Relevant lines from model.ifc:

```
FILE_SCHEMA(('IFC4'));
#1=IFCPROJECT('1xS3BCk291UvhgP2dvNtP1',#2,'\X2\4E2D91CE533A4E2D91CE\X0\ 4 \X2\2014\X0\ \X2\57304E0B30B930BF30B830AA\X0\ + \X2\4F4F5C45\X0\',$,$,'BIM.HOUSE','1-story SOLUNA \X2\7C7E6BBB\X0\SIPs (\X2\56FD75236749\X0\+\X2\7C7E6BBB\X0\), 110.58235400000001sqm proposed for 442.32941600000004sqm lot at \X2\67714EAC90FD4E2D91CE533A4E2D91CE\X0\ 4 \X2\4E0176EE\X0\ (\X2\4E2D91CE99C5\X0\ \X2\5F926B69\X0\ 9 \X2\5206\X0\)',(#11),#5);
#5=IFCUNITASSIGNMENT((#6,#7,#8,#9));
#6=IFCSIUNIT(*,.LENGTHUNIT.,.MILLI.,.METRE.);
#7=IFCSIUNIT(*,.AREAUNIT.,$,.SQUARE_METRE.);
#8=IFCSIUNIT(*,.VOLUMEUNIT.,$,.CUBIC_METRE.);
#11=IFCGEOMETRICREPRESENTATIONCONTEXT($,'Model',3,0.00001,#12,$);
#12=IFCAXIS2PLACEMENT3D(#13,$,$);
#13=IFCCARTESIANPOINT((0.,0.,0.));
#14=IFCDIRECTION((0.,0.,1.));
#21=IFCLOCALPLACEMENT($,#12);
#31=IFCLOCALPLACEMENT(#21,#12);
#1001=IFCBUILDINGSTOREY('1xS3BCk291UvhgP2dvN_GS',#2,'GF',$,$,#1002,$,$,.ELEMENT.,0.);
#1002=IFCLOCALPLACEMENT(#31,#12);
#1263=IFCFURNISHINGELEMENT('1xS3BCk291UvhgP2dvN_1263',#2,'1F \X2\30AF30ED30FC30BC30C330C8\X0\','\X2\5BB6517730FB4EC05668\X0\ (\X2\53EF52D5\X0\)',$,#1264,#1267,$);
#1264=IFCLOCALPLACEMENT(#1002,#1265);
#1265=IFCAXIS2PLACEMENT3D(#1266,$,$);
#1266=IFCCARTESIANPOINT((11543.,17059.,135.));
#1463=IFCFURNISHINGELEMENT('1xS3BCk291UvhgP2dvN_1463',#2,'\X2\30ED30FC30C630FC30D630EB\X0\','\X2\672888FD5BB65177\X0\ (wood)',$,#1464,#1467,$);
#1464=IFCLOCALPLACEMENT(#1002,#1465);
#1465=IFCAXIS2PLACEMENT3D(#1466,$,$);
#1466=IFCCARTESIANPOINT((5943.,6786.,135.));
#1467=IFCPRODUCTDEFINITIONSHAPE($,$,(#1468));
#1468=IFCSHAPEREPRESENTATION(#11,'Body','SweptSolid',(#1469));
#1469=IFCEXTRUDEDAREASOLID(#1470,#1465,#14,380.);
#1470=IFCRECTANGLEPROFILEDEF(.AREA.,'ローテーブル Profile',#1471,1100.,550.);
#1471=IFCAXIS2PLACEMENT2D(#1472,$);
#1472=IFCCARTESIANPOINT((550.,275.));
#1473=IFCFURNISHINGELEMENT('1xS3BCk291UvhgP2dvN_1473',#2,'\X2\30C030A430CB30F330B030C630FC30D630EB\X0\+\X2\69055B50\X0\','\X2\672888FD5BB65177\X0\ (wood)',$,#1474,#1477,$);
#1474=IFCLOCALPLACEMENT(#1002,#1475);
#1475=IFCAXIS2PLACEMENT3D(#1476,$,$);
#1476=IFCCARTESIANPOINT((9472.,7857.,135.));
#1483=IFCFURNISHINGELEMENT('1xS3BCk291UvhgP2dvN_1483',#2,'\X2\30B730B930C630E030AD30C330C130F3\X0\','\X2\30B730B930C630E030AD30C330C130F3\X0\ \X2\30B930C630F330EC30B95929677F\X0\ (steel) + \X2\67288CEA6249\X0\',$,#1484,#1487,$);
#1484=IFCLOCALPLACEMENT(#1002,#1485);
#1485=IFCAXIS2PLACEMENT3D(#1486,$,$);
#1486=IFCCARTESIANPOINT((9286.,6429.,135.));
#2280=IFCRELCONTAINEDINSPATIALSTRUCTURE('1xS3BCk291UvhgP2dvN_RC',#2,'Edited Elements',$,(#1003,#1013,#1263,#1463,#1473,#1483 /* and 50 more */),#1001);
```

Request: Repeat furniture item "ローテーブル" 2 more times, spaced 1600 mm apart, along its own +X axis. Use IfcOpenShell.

```python
import ifcopenshell
import ifcopenshell.api.geometry
import ifcopenshell.api.root
import ifcopenshell.util.element
import ifcopenshell.util.placement
import ifcopenshell.util.unit

model = ifcopenshell.open("model.ifc")
unit_scale = ifcopenshell.util.unit.calculate_unit_scale(model)


def reuse_history(source, copy):
    """copy_class also copies each property set's owner history, people and application; keep the originals."""
    for rel in copy.IsDefinedBy:
        if rel.is_a("IfcRelDefinesByProperties") and (history := rel.RelatingPropertyDefinition.OwnerHistory):
            rel.RelatingPropertyDefinition.OwnerHistory = source.OwnerHistory
            ifcopenshell.util.element.remove_deep2(model, history)


source = model.by_guid("1xS3BCk291UvhgP2dvN_1463")
base = ifcopenshell.util.placement.get_local_placement(source.ObjectPlacement)
step = base[:3, 0] * 1.6 / unit_scale

for i in range(1, 3):
    copy = ifcopenshell.api.root.copy_class(model, product=source)
    copy.Representation = ifcopenshell.util.element.copy_deep(
        model, source.Representation, exclude=["IfcGeometricRepresentationContext", "IfcRepresentationMap"]
    )
    reuse_history(source, copy)
    matrix = base.copy()
    matrix[:3, 3] += i * step
    print("added at", matrix[:3, 3].round(3) + 0.0)
    ifcopenshell.api.geometry.edit_object_placement(model, product=copy, matrix=matrix, is_si=False)

model.write("model-out.ifc")
```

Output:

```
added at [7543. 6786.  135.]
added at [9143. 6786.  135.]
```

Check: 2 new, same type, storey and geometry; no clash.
